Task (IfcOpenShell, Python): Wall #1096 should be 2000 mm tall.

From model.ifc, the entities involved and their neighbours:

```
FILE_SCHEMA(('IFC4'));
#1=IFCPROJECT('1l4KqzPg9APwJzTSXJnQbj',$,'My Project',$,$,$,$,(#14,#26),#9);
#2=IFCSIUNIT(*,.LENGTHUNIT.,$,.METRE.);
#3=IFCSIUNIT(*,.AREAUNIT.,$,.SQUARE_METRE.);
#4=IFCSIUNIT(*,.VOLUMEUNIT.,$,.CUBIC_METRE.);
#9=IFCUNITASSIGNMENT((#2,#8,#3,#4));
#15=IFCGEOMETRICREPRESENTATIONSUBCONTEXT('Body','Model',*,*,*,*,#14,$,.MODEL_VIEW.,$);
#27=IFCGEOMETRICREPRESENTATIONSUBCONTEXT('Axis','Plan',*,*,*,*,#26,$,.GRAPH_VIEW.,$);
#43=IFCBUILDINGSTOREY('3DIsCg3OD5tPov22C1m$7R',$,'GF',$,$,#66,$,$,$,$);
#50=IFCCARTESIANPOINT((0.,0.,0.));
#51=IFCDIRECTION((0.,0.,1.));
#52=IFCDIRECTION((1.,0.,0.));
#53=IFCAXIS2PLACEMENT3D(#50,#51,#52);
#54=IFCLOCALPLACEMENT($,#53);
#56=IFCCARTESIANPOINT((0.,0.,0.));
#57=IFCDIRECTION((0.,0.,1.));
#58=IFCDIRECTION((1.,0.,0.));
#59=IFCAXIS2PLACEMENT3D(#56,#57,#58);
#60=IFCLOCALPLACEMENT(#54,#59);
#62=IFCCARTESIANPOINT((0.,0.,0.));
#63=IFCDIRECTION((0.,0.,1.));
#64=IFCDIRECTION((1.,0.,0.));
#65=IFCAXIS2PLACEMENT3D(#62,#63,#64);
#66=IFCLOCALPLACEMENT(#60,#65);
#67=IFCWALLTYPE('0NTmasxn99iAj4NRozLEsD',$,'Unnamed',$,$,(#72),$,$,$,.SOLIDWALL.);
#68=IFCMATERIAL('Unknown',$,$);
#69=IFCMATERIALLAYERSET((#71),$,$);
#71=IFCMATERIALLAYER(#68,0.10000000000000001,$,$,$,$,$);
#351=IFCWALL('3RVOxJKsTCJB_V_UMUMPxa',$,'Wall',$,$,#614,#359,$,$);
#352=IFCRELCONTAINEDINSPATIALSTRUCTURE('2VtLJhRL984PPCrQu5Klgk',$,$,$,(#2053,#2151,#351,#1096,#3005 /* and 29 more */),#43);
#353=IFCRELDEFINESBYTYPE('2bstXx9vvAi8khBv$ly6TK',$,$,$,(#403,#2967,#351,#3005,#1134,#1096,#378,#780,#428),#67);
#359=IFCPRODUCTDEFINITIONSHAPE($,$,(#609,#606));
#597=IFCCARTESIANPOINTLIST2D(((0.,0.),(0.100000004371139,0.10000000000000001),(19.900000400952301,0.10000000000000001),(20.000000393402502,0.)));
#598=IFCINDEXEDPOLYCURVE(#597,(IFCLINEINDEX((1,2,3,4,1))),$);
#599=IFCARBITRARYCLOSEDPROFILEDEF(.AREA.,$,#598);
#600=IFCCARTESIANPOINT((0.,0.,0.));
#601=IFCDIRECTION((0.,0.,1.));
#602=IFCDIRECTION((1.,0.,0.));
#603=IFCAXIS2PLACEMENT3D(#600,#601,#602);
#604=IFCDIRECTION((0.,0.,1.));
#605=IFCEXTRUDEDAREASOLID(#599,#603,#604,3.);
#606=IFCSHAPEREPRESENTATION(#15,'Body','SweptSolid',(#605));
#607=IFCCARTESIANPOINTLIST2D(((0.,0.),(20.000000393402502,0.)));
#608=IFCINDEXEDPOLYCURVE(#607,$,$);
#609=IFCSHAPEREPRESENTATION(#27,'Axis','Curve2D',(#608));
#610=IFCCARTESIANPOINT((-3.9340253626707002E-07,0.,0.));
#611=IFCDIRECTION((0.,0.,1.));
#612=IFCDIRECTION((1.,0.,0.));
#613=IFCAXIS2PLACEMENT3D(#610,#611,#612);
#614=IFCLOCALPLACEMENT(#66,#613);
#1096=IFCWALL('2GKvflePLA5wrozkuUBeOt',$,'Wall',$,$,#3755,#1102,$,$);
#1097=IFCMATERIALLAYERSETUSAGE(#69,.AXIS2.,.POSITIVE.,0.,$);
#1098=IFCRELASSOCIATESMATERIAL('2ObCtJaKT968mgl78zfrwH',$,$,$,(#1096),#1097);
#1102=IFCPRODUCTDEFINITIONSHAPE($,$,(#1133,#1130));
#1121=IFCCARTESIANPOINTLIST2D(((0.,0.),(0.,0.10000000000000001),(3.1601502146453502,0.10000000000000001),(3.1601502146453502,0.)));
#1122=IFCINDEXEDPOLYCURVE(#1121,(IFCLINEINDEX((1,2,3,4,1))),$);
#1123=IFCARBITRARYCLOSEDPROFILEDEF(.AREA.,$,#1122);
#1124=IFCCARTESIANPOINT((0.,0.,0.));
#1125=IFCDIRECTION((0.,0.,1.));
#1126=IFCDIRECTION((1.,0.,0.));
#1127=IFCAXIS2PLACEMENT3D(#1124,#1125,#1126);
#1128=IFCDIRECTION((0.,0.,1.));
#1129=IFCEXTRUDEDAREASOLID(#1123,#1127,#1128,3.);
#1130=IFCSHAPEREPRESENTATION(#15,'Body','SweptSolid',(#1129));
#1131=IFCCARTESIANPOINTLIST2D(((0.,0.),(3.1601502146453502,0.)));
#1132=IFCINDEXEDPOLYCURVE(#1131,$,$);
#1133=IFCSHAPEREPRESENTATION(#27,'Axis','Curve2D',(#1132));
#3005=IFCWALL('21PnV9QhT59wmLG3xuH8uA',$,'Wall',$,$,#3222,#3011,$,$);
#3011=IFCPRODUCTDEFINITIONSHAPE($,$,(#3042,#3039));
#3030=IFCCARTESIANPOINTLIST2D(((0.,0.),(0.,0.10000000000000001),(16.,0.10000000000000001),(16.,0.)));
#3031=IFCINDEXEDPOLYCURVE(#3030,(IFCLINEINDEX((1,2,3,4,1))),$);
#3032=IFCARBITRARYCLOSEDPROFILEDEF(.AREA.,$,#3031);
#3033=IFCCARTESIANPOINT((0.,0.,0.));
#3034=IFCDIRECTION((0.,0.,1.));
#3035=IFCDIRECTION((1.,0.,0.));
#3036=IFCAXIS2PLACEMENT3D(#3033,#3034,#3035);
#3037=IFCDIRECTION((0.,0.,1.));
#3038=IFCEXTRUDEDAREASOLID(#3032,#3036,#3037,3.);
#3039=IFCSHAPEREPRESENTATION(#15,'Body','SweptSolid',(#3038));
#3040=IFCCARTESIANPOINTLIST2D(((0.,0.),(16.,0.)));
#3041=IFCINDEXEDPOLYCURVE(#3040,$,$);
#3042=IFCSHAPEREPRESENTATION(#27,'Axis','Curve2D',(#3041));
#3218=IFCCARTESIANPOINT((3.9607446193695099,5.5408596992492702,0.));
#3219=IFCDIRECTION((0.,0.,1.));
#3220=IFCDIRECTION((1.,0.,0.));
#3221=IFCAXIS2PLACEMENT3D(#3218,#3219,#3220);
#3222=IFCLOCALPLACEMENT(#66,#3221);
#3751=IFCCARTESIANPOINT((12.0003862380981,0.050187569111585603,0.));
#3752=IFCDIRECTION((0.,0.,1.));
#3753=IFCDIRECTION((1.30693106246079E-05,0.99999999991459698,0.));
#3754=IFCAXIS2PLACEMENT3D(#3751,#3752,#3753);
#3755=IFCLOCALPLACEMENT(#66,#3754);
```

```python
import ifcopenshell
import ifcopenshell.geom
import ifcopenshell.util.representation
import ifcopenshell.util.shape

model = ifcopenshell.open("model.ifc")
settings = ifcopenshell.geom.settings()


def volume(element):
    """Net volume in cubic metres, openings subtracted."""
    shape = ifcopenshell.geom.create_shape(settings, element)
    return ifcopenshell.util.shape.get_volume(shape.geometry)


wall = model.by_guid("2GKvflePLA5wrozkuUBeOt")
before = volume(wall)

body = ifcopenshell.util.representation.get_representation(wall, "Model", "Body")
solid = body.Items[0]
old_height = solid.Depth
solid.Depth = 2.0
after = volume(wall)

print(f"height {old_height:g} -> {solid.Depth:g}, volume {before:.3f} -> {after:.3f} m3")

model.write("model-out.ifc")
```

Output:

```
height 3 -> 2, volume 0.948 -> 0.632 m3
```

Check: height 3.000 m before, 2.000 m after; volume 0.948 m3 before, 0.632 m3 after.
